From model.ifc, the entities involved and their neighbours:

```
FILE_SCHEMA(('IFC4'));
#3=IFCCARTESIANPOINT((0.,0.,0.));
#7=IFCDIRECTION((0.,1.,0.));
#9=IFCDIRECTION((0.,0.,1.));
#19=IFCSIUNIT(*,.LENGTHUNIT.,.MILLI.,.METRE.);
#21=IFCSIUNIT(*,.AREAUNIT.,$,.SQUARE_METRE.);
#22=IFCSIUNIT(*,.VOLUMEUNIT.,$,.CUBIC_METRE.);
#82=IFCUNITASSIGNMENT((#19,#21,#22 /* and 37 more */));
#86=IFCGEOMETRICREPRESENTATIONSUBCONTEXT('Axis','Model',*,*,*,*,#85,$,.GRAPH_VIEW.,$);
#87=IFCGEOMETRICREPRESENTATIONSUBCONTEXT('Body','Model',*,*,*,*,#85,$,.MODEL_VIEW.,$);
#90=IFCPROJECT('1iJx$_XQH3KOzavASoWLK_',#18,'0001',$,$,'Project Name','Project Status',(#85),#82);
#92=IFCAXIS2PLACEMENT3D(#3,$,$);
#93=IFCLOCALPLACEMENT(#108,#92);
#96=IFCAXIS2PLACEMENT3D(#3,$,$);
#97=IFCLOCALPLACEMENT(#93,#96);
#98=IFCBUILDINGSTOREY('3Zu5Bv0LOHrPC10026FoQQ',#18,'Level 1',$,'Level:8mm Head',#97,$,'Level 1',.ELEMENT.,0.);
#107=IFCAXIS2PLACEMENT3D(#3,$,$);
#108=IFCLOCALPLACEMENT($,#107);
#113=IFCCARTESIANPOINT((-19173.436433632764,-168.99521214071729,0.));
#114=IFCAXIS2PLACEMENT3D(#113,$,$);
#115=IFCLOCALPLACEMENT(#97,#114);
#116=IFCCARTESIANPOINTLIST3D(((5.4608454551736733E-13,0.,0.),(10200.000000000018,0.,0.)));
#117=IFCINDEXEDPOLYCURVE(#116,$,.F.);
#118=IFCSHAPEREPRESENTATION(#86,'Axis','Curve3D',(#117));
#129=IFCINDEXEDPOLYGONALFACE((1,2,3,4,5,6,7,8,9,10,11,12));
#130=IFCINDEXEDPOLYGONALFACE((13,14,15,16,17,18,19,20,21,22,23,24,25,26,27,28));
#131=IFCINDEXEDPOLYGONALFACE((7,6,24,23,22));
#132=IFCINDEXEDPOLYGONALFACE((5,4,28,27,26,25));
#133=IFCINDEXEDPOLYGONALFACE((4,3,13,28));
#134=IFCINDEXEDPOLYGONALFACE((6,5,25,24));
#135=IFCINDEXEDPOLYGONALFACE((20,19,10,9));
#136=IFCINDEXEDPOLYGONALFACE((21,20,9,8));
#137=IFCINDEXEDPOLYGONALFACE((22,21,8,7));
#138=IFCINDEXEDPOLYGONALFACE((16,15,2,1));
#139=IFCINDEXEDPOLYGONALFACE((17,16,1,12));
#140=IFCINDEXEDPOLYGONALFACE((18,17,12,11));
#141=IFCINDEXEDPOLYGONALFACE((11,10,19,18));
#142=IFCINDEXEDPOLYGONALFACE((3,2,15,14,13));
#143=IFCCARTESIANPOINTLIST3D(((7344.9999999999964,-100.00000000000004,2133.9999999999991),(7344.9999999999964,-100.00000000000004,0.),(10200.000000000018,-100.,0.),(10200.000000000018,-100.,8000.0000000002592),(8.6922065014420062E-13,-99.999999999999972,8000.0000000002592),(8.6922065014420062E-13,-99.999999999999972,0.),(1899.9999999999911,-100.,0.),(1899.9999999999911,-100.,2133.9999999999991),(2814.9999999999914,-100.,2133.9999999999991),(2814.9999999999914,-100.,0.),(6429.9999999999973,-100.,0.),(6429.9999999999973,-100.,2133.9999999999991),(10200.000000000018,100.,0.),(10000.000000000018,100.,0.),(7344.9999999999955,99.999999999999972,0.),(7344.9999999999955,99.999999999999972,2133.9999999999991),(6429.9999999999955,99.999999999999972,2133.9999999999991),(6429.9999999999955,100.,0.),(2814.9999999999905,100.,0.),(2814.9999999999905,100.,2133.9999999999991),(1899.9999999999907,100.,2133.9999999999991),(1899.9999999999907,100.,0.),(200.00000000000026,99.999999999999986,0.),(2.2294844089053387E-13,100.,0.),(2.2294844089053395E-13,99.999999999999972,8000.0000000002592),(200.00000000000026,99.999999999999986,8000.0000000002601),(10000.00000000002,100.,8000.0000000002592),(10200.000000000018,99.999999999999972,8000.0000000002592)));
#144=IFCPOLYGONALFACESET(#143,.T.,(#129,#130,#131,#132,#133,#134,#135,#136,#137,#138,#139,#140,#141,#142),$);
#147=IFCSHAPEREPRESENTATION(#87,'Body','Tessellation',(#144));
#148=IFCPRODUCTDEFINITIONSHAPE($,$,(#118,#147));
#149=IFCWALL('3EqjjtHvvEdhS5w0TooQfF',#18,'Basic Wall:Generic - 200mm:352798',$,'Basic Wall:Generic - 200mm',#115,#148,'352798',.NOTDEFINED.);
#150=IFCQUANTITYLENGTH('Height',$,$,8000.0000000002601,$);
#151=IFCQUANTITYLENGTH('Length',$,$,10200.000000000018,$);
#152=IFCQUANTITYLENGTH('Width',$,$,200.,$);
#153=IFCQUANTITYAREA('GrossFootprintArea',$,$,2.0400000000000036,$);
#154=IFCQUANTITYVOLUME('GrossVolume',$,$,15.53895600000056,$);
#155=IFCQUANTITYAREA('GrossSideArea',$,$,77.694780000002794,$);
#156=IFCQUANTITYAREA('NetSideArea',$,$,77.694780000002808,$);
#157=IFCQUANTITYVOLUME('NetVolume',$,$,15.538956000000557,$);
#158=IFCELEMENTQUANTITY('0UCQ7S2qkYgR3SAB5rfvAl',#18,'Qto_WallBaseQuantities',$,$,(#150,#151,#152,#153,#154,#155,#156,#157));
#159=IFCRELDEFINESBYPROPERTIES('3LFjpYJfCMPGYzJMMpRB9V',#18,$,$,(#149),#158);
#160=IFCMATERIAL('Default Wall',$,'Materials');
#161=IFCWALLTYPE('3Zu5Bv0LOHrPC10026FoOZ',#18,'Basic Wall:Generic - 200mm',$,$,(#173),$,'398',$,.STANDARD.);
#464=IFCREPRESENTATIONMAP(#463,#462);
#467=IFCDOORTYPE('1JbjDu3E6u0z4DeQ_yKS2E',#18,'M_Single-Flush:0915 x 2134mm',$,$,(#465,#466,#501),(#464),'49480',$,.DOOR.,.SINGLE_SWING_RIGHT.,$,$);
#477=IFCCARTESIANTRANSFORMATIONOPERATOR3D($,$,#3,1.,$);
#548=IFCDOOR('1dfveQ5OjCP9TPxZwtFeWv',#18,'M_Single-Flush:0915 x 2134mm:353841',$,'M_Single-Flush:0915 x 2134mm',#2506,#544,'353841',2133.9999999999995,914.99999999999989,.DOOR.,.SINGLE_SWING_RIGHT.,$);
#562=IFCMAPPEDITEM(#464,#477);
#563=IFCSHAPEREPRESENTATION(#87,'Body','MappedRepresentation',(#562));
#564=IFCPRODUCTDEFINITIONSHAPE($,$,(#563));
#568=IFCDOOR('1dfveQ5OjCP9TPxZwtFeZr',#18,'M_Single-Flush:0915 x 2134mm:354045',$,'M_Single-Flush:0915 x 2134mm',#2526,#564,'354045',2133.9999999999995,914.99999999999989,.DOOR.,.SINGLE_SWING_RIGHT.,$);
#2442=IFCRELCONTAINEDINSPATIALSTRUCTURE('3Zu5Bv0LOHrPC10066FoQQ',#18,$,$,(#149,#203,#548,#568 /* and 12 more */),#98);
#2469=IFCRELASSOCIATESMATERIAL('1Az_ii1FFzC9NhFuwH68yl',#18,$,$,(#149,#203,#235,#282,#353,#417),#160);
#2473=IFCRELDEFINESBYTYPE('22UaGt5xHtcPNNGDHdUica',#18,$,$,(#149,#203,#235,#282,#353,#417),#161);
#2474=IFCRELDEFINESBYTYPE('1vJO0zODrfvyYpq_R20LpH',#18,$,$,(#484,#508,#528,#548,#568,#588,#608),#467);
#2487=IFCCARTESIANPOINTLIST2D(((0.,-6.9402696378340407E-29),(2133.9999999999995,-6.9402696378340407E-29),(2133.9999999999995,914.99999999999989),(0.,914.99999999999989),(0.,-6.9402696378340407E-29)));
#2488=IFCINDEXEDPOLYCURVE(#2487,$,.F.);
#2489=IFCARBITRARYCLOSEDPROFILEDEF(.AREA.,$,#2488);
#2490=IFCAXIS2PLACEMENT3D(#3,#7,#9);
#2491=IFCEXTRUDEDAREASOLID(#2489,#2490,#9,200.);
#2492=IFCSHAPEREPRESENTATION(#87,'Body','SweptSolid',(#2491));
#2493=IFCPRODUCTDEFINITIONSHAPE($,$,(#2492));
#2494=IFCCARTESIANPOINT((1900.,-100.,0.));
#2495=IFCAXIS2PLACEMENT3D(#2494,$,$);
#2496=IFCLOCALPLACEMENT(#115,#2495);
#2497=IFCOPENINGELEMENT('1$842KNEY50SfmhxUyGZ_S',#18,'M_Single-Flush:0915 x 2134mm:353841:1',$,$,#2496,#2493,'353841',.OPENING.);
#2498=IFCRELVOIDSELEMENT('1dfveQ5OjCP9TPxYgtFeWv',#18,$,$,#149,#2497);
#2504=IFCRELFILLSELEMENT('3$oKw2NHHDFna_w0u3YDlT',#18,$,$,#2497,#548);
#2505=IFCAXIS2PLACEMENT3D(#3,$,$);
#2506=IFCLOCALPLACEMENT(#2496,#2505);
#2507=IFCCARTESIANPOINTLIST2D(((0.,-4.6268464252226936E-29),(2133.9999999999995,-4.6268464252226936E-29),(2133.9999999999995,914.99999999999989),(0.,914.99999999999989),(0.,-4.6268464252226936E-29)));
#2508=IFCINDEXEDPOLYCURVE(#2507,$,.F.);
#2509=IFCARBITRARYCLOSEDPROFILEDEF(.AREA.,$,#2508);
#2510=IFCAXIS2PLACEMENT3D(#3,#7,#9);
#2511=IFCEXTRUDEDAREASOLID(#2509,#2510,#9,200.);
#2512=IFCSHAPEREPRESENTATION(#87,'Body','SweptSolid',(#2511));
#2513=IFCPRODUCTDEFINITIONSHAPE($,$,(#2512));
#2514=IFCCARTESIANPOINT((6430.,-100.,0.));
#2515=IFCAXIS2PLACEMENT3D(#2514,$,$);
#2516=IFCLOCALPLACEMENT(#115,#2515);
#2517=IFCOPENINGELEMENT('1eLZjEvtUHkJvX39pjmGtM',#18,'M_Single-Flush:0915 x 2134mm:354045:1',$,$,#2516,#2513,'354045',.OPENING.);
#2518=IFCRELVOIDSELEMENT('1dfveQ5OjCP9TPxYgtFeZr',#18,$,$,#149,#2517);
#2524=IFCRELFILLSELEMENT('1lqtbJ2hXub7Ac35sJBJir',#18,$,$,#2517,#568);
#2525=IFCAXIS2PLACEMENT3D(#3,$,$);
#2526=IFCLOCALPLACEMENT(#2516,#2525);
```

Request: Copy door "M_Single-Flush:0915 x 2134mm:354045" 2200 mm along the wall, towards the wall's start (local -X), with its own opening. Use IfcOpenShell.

```python
import ifcopenshell
import ifcopenshell.api.feature
import ifcopenshell.api.geometry
import ifcopenshell.api.pset
import ifcopenshell.api.root
import ifcopenshell.geom
import ifcopenshell.util.element
import ifcopenshell.util.placement
import ifcopenshell.util.shape
import ifcopenshell.util.unit

model = ifcopenshell.open("model.ifc")
area_scale = ifcopenshell.util.unit.calculate_unit_scale(model, "AREAUNIT")
volume_scale = ifcopenshell.util.unit.calculate_unit_scale(model, "VOLUMEUNIT")
settings = ifcopenshell.geom.settings()


def volume(element):
    """Net volume in cubic metres, openings subtracted."""
    shape = ifcopenshell.geom.create_shape(settings, element)
    return ifcopenshell.util.shape.get_volume(shape.geometry)


def reuse_history(source, copy):
    """copy_class also copies each property set's owner history, people and application; keep the originals."""
    for rel in copy.IsDefinedBy:
        if rel.is_a("IfcRelDefinesByProperties") and (history := rel.RelatingPropertyDefinition.OwnerHistory):
            rel.RelatingPropertyDefinition.OwnerHistory = source.OwnerHistory
            ifcopenshell.util.element.remove_deep2(model, history)


door = model.by_id(568)
opening = door.FillsVoids[0].RelatingOpeningElement
wall = opening.VoidsElements[0].RelatingBuildingElement
before = volume(wall)
shift = ifcopenshell.util.placement.get_local_placement(wall.ObjectPlacement)[:3, 0] * -2200.0

# copy_class copies the void relationship, type, container and properties, but no geometry.
new_opening = ifcopenshell.api.root.copy_class(model, product=opening)
new_opening.Representation = ifcopenshell.util.element.copy_deep(
    model, opening.Representation, exclude=["IfcGeometricRepresentationContext", "IfcRepresentationMap"]
)
new_opening.Name = "M_Single-Flush:0915 x 2134mm"
new_opening.Tag = None
reuse_history(opening, new_opening)
new_door = ifcopenshell.api.root.copy_class(model, product=door)
new_door.Representation = ifcopenshell.util.element.copy_deep(
    model, door.Representation, exclude=["IfcGeometricRepresentationContext", "IfcRepresentationMap"]
)
new_door.Name = "M_Single-Flush:0915 x 2134mm"
new_door.Tag = None
reuse_history(door, new_door)
ifcopenshell.api.feature.add_filling(model, opening=new_opening, element=new_door)

for old, new in ((opening, new_opening), (door, new_door)):
    matrix = ifcopenshell.util.placement.get_local_placement(old.ObjectPlacement)
    matrix[:3, 3] += shift
    ifcopenshell.api.geometry.edit_object_placement(model, product=new, matrix=matrix, is_si=False)

after = volume(wall)
thickness = 0.2  # wall thickness in metres

# Update the wall's stored quantities.
qto = model.by_id(ifcopenshell.util.element.get_pset(wall, "Qto_WallBaseQuantities", should_inherit=False)["id"])
ifcopenshell.api.pset.edit_qto(model, qto=qto, properties={
    "NetSideArea": after / thickness / area_scale,
    "NetVolume": after / volume_scale,
})

print(f"wall volume {before:.3f} -> {after:.3f} m3")

model.write("model_updated.ifc")
```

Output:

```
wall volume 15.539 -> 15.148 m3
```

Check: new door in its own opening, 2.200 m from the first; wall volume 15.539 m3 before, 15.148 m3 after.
